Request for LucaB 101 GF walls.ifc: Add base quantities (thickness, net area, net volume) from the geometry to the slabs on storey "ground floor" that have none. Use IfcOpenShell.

First a look at what the model holds.

```python
import ifcopenshell
import ifcopenshell.util.element
import ifcopenshell.util.unit

model = ifcopenshell.open("LucaB 101 GF walls.ifc")
print(model.schema)
for unit_type in ("LENGTHUNIT", "AREAUNIT", "VOLUMEUNIT"):
    print(unit_type, ifcopenshell.util.unit.calculate_unit_scale(model, unit_type))
storey = next(s for s in model.by_type("IfcBuildingStorey") if s.Name == "ground floor")
slabs = [e for e in ifcopenshell.util.element.get_decomposition(storey) if e.is_a("IfcSlab")]
for e in sorted(slabs, key=lambda e: e.id()):
    print(e.id(), e.is_a(), e.Name, list(ifcopenshell.util.element.get_psets(e, qtos_only=True)), sep=" | ")
```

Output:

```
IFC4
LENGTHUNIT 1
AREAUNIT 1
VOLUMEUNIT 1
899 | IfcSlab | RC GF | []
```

```python
import ifcopenshell
import ifcopenshell.api.pset
import ifcopenshell.geom
import ifcopenshell.util.element
import ifcopenshell.util.shape
import ifcopenshell.util.unit

model = ifcopenshell.open("LucaB 101 GF walls.ifc")
unit_scale = ifcopenshell.util.unit.calculate_unit_scale(model)
area_scale = ifcopenshell.util.unit.calculate_unit_scale(model, "AREAUNIT")
volume_scale = ifcopenshell.util.unit.calculate_unit_scale(model, "VOLUMEUNIT")
settings = ifcopenshell.geom.settings()

storey = next(s for s in model.by_type("IfcBuildingStorey") if s.Name == "ground floor")
slabs = [e for e in ifcopenshell.util.element.get_decomposition(storey) if e.is_a("IfcSlab")]

for e in sorted(slabs, key=lambda e: e.id()):
    if ifcopenshell.util.element.get_psets(e, qtos_only=True, should_inherit=False):
        continue
    # Geometry comes back in metres, in the element's own axes.
    shape = ifcopenshell.geom.create_shape(settings, e)
    values = {
        "Width": ifcopenshell.util.shape.get_z(shape.geometry) / unit_scale,
        "NetArea": ifcopenshell.util.shape.get_footprint_area(shape.geometry) / area_scale,
        "NetVolume": ifcopenshell.util.shape.get_volume(shape.geometry) / volume_scale,
    }
    qto = ifcopenshell.api.pset.add_qto(model, product=e, name="Qto_SlabBaseQuantities")
    ifcopenshell.api.pset.edit_qto(model, qto=qto, properties=values)
    print(e.id(), {k: round(v, 3) for k, v in values.items()})

model.write("LucaB 101 GF walls_updated.ifc")
```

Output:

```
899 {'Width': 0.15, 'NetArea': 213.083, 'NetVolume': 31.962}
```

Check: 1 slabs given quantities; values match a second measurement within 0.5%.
